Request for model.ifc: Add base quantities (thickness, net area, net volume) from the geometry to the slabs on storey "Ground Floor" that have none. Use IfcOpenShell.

First a look at what the model holds.

```python
import ifcopenshell
import ifcopenshell.util.element
import ifcopenshell.util.unit

model = ifcopenshell.open("model.ifc")
print(model.schema)
for unit_type in ("LENGTHUNIT", "AREAUNIT", "VOLUMEUNIT"):
    print(unit_type, ifcopenshell.util.unit.calculate_unit_scale(model, unit_type))
storey = next(s for s in model.by_type("IfcBuildingStorey") if s.Name == "Ground Floor")
slabs = [e for e in ifcopenshell.util.element.get_decomposition(storey) if e.is_a("IfcSlab")]
for e in sorted(slabs, key=lambda e: e.id()):
    print(e.id(), e.is_a(), e.Name, list(ifcopenshell.util.element.get_psets(e, qtos_only=True)), sep=" | ")
```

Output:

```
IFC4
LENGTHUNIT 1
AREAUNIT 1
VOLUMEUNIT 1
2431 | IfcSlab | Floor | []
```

```python
import ifcopenshell
import ifcopenshell.api.pset
import ifcopenshell.geom
import ifcopenshell.util.element
import ifcopenshell.util.shape
import ifcopenshell.util.unit

model = ifcopenshell.open("model.ifc")
unit_scale = ifcopenshell.util.unit.calculate_unit_scale(model)
area_scale = ifcopenshell.util.unit.calculate_unit_scale(model, "AREAUNIT")
volume_scale = ifcopenshell.util.unit.calculate_unit_scale(model, "VOLUMEUNIT")
settings = ifcopenshell.geom.settings()

storey = next(s for s in model.by_type("IfcBuildingStorey") if s.Name == "Ground Floor")
slabs = [e for e in ifcopenshell.util.element.get_decomposition(storey) if e.is_a("IfcSlab")]

for e in sorted(slabs, key=lambda e: e.id()):
    if ifcopenshell.util.element.get_psets(e, qtos_only=True, should_inherit=False):
        continue
    # Geometry comes back in metres, in the element's own axes.
    shape = ifcopenshell.geom.create_shape(settings, e)
    values = {
        "Width": ifcopenshell.util.shape.get_z(shape.geometry) / unit_scale,
        "NetArea": ifcopenshell.util.shape.get_footprint_area(shape.geometry) / area_scale,
        "NetVolume": ifcopenshell.util.shape.get_volume(shape.geometry) / volume_scale,
    }
    qto = ifcopenshell.api.pset.add_qto(model, product=e, name="Qto_SlabBaseQuantities")
    ifcopenshell.api.pset.edit_qto(model, qto=qto, properties=values)
    print(e.id(), {k: round(v, 3) for k, v in values.items()})

model.write("model_edited.ifc")
```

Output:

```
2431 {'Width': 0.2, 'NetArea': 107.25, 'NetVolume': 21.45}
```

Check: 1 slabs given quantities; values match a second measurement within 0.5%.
